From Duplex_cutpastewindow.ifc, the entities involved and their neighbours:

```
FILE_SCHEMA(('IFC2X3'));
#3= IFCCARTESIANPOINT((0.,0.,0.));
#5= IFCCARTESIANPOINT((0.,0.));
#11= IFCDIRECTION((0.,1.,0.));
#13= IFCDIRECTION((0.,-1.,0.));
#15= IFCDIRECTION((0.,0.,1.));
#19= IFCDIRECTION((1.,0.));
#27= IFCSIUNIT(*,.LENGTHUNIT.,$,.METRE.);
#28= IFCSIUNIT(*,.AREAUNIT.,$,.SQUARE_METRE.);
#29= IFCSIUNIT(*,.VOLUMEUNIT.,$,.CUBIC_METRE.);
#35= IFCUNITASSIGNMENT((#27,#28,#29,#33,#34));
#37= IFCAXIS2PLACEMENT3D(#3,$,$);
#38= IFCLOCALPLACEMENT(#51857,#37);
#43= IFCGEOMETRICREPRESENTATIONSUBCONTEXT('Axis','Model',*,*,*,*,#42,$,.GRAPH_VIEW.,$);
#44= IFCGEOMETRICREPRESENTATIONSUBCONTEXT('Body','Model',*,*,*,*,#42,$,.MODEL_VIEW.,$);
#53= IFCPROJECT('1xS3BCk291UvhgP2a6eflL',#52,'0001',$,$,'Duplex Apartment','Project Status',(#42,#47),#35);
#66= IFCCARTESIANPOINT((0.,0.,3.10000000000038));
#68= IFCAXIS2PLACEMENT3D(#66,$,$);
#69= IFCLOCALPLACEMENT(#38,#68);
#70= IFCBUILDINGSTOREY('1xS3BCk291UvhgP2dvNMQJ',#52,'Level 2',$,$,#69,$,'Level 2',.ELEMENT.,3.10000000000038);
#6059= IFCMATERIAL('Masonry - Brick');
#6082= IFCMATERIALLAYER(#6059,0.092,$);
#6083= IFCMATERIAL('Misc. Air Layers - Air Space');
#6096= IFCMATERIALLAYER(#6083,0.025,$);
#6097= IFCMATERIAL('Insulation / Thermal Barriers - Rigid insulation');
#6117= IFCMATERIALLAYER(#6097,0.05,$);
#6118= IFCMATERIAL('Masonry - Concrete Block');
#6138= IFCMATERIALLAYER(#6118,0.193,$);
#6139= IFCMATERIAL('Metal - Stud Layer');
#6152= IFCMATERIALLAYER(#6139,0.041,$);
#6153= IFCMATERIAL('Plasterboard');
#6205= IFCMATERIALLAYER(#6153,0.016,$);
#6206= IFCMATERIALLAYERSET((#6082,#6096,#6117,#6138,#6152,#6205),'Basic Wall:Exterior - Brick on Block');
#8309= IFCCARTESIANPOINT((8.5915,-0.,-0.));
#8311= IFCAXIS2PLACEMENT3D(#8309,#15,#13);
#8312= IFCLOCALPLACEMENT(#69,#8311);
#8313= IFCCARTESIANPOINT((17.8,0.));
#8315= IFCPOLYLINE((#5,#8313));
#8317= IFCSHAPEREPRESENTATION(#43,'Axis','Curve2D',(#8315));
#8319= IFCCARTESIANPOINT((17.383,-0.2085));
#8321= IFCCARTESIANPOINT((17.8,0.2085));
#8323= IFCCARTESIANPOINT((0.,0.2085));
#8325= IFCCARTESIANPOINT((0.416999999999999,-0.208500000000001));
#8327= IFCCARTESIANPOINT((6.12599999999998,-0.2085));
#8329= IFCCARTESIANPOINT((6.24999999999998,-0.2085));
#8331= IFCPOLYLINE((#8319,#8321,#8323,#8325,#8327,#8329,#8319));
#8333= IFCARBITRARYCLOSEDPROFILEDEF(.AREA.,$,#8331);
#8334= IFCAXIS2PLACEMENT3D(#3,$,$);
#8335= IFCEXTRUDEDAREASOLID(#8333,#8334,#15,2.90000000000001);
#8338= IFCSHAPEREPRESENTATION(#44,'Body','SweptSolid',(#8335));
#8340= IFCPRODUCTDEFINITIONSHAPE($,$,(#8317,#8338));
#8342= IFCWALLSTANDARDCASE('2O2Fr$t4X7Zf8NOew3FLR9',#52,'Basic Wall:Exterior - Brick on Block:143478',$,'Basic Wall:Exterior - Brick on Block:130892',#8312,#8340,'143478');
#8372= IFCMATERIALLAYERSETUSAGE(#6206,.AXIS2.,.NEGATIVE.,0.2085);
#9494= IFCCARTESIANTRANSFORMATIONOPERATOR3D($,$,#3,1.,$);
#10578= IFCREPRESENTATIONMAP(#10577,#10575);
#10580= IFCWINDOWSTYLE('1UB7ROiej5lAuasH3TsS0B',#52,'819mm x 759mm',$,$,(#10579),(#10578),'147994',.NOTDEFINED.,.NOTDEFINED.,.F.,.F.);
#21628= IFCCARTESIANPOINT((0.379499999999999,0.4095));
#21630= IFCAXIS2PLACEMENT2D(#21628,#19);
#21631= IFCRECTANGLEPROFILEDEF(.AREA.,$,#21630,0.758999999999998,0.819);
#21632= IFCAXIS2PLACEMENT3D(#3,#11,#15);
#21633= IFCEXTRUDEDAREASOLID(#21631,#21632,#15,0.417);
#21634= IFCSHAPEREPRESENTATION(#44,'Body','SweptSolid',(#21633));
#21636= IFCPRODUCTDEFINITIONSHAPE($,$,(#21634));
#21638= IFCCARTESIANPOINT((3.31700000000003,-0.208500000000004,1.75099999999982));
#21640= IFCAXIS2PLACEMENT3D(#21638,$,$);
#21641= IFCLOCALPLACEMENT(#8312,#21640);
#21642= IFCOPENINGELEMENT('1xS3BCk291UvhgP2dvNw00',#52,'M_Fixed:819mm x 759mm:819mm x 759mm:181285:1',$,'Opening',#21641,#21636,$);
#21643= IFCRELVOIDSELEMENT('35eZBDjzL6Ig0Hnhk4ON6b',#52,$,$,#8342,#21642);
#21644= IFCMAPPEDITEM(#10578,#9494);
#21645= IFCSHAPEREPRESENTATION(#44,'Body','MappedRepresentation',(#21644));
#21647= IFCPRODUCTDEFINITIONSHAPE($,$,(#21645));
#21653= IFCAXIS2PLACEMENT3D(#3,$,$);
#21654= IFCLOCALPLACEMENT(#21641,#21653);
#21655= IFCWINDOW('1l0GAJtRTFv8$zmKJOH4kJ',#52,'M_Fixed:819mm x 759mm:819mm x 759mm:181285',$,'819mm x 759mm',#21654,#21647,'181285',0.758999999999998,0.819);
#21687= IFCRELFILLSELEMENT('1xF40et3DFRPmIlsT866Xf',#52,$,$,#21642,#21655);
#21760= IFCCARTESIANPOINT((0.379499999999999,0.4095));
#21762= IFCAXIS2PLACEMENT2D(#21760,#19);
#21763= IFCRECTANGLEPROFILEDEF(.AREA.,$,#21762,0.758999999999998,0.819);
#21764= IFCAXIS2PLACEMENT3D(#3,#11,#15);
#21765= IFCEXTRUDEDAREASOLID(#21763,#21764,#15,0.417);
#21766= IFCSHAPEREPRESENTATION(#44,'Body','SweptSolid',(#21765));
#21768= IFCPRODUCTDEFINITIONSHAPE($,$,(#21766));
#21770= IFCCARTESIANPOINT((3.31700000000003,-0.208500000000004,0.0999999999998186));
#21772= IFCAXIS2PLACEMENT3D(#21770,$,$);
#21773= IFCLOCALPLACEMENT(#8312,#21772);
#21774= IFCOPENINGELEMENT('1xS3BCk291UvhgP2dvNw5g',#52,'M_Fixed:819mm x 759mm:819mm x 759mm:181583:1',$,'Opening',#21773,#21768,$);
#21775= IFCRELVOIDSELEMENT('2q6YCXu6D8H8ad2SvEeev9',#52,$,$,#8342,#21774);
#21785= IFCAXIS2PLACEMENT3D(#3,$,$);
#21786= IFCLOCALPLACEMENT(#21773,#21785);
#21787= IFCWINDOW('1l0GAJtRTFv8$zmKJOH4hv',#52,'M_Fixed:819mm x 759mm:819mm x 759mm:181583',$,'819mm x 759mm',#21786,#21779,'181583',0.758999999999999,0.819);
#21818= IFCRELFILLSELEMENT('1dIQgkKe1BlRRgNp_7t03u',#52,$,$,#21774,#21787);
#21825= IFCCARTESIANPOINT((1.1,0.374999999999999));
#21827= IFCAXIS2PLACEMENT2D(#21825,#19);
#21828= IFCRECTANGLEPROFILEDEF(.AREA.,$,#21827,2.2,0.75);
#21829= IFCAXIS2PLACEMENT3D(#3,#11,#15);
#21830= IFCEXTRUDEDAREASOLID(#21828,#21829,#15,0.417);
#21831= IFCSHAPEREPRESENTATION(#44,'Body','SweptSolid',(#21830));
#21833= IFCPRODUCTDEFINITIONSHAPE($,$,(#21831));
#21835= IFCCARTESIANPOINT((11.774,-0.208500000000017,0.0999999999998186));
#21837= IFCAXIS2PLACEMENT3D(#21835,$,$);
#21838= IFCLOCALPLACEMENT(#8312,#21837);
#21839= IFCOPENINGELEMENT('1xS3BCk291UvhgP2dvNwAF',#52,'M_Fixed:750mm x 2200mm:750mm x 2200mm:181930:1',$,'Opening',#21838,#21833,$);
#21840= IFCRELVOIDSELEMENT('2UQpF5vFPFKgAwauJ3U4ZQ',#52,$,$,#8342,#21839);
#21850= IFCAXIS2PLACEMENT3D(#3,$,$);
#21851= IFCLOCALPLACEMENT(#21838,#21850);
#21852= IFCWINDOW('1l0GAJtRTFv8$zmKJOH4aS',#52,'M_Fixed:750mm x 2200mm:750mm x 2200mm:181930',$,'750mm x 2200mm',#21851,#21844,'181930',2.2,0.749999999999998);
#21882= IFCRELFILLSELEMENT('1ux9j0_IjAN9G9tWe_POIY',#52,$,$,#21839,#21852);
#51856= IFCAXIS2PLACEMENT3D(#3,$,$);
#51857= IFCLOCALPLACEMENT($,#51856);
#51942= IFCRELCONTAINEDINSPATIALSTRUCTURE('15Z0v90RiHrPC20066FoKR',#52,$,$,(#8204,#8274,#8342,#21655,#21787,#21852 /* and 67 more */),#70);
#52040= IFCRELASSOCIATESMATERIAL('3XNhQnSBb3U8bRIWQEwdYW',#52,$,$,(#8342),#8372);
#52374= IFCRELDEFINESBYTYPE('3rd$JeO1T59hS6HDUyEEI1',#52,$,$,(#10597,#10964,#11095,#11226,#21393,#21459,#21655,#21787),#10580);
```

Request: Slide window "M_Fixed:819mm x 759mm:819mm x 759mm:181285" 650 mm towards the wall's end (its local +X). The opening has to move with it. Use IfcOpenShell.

```python
import ifcopenshell
import ifcopenshell.api.geometry
import ifcopenshell.util.placement
import ifcopenshell.util.unit

model = ifcopenshell.open("Duplex_cutpastewindow.ifc")
unit_scale = ifcopenshell.util.unit.calculate_unit_scale(model)

window = model.by_guid("1l0GAJtRTFv8$zmKJOH4kJ")
opening = window.FillsVoids[0].RelatingOpeningElement
wall = opening.VoidsElements[0].RelatingBuildingElement

wall_matrix = ifcopenshell.util.placement.get_local_placement(wall.ObjectPlacement)
shift = wall_matrix[:3, 0] * 0.65 / unit_scale
before = ifcopenshell.util.placement.get_local_placement(window.ObjectPlacement)[:3, 3].copy()

# The window is placed relative to its opening, so it follows when the opening moves.
matrix = ifcopenshell.util.placement.get_local_placement(opening.ObjectPlacement)
matrix[:3, 3] += shift
ifcopenshell.api.geometry.edit_object_placement(
    model, product=opening, matrix=matrix, is_si=False, should_transform_children=True
)

after = ifcopenshell.util.placement.get_local_placement(window.ObjectPlacement)[:3, 3]
print("window moved by", (after - before).round(3) + 0.0)

model.write("Duplex_cutpastewindow_rev.ifc")
```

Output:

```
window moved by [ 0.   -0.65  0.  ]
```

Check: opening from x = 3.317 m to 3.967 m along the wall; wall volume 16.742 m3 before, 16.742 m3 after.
